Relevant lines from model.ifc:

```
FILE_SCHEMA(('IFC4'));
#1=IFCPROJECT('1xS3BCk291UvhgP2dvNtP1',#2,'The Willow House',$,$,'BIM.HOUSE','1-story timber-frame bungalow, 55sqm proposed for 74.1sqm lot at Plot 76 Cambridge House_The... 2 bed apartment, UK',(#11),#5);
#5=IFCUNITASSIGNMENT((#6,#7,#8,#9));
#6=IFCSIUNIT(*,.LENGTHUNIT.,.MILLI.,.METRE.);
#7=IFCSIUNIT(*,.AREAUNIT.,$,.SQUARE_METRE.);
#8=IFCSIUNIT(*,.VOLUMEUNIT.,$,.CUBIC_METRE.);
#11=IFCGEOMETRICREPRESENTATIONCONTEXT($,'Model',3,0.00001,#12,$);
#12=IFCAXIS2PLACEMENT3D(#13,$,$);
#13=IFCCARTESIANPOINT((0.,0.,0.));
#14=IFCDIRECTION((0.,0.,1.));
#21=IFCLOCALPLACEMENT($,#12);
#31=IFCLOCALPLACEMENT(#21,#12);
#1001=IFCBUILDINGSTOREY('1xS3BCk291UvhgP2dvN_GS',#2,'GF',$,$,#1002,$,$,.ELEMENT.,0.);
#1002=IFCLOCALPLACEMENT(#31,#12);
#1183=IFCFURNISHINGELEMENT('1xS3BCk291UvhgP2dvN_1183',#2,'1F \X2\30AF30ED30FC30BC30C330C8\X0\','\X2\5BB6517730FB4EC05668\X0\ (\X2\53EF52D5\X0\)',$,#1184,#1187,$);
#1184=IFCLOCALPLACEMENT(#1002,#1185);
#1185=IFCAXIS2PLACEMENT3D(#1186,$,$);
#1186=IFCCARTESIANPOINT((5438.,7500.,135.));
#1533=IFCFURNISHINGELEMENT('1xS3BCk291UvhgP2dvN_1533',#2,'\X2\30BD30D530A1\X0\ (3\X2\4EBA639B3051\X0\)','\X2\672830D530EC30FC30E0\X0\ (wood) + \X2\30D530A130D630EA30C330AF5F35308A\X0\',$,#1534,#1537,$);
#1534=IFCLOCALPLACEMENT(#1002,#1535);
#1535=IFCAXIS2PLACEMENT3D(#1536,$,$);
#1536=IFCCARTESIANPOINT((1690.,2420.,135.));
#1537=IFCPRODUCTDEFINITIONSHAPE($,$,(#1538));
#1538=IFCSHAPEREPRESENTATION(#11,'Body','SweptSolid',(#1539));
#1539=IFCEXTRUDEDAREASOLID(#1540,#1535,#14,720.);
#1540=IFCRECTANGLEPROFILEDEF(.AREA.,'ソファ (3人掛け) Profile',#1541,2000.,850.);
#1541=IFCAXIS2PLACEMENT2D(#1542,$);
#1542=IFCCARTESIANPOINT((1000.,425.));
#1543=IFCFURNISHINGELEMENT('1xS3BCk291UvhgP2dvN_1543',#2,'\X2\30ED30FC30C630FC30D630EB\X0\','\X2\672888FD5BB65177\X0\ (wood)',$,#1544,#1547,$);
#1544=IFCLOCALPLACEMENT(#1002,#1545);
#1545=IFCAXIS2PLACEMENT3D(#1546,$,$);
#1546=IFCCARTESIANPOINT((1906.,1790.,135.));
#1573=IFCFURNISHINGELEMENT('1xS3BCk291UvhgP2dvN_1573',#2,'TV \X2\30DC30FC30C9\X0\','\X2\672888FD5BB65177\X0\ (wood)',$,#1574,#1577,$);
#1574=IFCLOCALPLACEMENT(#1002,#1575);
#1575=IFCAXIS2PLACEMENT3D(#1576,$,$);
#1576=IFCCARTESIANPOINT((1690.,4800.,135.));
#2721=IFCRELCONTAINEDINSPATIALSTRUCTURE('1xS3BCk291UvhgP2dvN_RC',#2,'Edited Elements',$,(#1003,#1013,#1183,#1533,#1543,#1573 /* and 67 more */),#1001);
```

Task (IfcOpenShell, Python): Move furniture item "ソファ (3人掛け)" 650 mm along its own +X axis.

```python
import ifcopenshell
import ifcopenshell.api.geometry
import ifcopenshell.util.placement

model = ifcopenshell.open("model.ifc")

item = model.by_guid("1xS3BCk291UvhgP2dvN_1533")
matrix = ifcopenshell.util.placement.get_local_placement(item.ObjectPlacement)
matrix[:3, 3] += matrix[:3, 0] * 650.0
ifcopenshell.api.geometry.edit_object_placement(model, product=item, matrix=matrix, is_si=False)

print(ifcopenshell.util.placement.get_local_placement(item.ObjectPlacement).round(3) + 0.0)

model.write("model-out.ifc")
```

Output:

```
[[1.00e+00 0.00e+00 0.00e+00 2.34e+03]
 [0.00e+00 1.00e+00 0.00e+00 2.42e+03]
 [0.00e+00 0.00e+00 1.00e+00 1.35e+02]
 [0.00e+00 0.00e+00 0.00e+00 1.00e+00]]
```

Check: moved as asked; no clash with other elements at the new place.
